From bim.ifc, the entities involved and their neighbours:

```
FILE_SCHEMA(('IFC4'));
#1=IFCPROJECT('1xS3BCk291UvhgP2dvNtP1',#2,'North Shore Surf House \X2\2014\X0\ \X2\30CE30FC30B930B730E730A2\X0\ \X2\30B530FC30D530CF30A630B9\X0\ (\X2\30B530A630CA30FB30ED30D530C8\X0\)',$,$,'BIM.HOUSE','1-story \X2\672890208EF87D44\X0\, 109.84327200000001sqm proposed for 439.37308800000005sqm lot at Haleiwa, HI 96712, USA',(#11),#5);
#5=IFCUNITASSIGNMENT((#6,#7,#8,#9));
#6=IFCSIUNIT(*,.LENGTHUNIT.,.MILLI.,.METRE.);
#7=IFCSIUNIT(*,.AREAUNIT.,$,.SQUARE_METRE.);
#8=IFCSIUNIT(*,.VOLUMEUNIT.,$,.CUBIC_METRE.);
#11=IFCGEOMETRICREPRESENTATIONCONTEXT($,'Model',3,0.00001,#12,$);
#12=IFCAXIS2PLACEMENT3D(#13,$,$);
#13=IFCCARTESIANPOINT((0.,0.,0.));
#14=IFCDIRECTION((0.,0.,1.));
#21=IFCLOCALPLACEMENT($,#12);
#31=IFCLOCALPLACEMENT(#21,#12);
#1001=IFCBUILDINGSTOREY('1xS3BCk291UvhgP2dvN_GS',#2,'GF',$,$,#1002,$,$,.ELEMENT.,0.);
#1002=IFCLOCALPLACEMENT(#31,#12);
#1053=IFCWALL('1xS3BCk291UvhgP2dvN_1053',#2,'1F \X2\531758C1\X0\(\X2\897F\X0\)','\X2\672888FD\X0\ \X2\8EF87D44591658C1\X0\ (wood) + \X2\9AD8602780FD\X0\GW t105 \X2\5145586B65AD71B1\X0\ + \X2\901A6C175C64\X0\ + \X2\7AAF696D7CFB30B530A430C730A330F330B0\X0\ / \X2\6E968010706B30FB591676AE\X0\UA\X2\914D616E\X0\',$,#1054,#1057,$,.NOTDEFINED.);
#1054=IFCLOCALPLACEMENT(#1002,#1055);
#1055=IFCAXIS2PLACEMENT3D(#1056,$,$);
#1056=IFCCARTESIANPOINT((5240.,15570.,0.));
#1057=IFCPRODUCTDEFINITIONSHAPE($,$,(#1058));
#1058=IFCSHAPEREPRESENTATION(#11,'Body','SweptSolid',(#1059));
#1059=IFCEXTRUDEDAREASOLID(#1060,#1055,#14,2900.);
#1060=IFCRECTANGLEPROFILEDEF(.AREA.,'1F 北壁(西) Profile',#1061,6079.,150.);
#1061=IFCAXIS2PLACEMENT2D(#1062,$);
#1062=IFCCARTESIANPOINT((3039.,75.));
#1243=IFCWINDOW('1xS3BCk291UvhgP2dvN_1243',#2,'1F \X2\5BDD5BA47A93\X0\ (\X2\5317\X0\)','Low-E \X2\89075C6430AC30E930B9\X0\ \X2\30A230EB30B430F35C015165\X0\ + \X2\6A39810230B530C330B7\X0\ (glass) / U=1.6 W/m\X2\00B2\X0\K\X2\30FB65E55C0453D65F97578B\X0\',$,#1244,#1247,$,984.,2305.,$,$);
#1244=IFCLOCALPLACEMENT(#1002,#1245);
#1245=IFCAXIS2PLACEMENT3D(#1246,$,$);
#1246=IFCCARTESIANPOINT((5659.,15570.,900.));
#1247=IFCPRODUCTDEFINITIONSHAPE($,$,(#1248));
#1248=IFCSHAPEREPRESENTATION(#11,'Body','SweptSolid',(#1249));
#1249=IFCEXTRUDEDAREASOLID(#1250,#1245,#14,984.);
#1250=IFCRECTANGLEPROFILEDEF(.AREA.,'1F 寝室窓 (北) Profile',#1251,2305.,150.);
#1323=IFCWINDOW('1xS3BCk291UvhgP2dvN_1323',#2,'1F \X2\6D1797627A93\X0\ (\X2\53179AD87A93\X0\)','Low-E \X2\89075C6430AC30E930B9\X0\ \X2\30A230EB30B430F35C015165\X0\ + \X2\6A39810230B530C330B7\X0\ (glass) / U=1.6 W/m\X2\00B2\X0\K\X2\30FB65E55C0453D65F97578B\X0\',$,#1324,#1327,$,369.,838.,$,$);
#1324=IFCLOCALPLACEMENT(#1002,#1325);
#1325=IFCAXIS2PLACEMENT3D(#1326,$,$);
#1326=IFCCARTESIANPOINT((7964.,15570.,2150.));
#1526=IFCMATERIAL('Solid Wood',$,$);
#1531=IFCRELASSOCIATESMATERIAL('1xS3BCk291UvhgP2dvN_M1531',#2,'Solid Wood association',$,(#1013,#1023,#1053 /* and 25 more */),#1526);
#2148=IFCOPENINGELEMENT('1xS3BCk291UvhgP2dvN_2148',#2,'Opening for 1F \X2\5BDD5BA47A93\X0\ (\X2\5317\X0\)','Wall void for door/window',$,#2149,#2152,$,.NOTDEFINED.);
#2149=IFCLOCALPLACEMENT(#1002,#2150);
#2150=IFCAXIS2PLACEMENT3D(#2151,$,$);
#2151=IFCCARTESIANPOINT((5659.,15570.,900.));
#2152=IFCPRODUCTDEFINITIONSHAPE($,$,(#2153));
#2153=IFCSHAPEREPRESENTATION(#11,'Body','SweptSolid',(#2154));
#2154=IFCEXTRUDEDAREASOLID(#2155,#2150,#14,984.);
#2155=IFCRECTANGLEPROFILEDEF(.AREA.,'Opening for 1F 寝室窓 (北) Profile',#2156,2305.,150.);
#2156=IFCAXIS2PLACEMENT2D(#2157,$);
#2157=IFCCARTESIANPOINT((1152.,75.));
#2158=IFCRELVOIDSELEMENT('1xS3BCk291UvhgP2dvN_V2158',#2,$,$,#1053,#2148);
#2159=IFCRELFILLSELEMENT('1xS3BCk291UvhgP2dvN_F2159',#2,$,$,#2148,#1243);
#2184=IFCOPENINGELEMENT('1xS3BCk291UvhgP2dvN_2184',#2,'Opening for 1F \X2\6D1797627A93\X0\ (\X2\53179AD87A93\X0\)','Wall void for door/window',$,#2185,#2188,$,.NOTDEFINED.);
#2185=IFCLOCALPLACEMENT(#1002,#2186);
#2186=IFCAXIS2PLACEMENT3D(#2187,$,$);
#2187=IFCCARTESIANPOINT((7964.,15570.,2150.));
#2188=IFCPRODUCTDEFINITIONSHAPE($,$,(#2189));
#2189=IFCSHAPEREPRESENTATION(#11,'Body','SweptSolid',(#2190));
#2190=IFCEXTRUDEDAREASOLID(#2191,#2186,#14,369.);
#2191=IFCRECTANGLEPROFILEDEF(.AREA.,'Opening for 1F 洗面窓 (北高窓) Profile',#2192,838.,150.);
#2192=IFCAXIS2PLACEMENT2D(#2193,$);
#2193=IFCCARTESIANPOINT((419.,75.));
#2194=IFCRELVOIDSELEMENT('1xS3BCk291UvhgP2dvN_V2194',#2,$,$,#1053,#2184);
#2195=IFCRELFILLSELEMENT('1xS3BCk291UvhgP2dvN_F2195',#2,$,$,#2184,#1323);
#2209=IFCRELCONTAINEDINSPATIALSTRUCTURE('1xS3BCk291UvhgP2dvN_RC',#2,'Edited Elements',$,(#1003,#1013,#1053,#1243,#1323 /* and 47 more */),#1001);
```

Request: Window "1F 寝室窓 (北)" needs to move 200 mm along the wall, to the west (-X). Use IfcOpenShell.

```python
import ifcopenshell
import ifcopenshell.api.geometry
import ifcopenshell.util.placement
import ifcopenshell.util.unit

model = ifcopenshell.open("bim.ifc")
unit_scale = ifcopenshell.util.unit.calculate_unit_scale(model)

window = model.by_guid("1xS3BCk291UvhgP2dvN_1243")
opening = window.FillsVoids[0].RelatingOpeningElement
wall = opening.VoidsElements[0].RelatingBuildingElement

wall_matrix = ifcopenshell.util.placement.get_local_placement(wall.ObjectPlacement)
shift = wall_matrix[:3, 0] * -0.2 / unit_scale
before = ifcopenshell.util.placement.get_local_placement(window.ObjectPlacement)[:3, 3].copy()

# The window is not placed relative to its opening, so move both.
for product in (opening, window):
    matrix = ifcopenshell.util.placement.get_local_placement(product.ObjectPlacement)
    matrix[:3, 3] += shift
    ifcopenshell.api.geometry.edit_object_placement(model, product=product, matrix=matrix, is_si=False)

after = ifcopenshell.util.placement.get_local_placement(window.ObjectPlacement)[:3, 3]
print("window moved by", (after - before).round(3) + 0.0)

model.write("bim-out.ifc")
```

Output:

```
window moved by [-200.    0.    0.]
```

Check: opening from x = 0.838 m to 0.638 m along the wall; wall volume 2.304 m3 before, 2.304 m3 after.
